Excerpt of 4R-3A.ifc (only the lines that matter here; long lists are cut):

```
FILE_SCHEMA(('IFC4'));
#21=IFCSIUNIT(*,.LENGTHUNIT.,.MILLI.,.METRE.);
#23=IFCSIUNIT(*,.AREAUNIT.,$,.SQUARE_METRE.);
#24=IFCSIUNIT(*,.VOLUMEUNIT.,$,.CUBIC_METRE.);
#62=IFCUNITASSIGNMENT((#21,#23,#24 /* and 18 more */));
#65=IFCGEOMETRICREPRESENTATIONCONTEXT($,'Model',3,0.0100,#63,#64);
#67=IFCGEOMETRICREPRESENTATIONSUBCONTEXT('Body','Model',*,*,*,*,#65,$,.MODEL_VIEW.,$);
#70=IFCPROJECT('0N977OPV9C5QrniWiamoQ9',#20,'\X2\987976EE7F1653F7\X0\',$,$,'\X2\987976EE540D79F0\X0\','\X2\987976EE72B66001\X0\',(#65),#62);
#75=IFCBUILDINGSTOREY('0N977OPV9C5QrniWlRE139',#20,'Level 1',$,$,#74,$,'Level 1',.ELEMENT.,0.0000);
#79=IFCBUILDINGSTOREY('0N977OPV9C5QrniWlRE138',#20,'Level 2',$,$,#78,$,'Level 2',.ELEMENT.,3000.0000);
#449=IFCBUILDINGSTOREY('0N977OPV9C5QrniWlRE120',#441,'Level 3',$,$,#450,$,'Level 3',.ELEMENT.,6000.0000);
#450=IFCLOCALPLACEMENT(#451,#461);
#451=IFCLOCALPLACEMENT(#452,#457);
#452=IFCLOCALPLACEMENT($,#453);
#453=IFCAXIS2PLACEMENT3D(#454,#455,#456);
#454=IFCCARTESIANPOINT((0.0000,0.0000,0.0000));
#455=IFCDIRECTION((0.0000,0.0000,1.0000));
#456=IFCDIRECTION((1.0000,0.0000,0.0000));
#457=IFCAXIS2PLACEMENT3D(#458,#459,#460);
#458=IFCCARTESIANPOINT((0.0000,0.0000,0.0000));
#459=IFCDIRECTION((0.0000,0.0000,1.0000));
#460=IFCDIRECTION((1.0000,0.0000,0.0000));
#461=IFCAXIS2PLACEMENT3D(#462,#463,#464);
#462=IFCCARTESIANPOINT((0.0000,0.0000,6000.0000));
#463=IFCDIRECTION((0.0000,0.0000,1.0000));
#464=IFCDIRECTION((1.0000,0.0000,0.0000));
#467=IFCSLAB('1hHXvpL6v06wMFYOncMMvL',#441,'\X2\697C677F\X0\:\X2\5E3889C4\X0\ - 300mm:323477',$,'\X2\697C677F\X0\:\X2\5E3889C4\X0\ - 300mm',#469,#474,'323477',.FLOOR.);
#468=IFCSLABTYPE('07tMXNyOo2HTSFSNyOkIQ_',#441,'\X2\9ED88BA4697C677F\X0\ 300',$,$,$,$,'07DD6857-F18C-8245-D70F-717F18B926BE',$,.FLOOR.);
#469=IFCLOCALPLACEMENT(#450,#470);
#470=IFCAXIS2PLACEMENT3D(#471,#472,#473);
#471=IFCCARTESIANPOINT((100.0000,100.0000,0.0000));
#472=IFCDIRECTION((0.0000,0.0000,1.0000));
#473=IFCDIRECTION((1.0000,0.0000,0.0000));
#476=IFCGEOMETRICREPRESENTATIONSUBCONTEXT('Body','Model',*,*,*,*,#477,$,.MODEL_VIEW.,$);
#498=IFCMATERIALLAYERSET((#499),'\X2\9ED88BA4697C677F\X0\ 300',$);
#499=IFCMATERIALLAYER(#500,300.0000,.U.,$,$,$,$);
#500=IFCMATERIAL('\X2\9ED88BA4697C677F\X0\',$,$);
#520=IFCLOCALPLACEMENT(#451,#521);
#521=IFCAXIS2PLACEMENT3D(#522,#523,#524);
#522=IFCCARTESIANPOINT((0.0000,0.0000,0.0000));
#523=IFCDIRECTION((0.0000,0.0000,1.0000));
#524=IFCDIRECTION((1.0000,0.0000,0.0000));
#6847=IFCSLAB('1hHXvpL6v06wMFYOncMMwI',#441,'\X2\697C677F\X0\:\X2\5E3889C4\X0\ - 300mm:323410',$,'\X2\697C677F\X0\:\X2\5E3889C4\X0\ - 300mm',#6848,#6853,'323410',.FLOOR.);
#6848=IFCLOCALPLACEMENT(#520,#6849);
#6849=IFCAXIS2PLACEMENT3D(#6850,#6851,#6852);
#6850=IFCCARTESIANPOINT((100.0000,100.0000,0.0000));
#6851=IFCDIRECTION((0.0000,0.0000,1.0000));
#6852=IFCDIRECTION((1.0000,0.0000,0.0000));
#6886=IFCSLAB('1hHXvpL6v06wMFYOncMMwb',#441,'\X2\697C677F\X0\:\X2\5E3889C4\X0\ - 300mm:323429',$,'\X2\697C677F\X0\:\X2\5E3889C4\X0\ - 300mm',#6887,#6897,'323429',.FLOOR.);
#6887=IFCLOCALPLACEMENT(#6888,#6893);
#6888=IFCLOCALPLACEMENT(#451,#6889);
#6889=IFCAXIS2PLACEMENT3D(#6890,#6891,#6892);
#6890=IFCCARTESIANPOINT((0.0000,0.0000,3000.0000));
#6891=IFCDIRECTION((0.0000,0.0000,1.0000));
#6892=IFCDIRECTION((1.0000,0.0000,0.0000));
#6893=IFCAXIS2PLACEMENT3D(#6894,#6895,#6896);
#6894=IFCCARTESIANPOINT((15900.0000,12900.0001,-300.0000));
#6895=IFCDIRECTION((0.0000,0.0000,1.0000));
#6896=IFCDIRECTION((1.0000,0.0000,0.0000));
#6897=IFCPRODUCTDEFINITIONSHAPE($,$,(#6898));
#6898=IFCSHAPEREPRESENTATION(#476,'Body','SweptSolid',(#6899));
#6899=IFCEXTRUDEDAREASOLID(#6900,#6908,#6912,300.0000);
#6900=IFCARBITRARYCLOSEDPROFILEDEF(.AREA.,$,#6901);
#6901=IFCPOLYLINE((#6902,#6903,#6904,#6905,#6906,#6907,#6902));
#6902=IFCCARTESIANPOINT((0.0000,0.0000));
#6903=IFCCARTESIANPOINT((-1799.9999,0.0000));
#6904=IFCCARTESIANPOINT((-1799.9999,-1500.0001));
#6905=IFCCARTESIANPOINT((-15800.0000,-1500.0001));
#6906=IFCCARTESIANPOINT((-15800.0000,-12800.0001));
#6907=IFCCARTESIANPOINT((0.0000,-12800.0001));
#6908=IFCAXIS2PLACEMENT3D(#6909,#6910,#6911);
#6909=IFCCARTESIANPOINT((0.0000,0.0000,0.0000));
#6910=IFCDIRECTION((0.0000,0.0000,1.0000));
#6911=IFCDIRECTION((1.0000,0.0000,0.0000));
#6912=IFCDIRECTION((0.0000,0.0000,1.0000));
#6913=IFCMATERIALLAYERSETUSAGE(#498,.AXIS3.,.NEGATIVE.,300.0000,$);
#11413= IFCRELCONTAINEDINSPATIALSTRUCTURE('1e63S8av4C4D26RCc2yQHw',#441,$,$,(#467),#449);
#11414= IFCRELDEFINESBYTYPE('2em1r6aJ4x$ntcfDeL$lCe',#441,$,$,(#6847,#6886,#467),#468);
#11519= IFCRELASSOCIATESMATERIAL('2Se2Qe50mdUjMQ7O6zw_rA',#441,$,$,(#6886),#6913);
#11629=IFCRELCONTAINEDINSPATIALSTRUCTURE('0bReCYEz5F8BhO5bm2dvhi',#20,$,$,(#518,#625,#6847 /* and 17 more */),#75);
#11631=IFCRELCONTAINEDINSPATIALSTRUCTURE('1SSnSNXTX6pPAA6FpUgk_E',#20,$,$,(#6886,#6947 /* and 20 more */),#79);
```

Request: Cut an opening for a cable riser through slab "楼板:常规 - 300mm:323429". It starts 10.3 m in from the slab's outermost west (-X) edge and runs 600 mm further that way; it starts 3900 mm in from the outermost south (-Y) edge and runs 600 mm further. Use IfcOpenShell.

```python
import numpy as np
import ifcopenshell
import ifcopenshell.api.feature
import ifcopenshell.api.geometry
import ifcopenshell.api.root
import ifcopenshell.geom
import ifcopenshell.util.placement
import ifcopenshell.util.representation
import ifcopenshell.util.shape
import ifcopenshell.util.unit

model = ifcopenshell.open("4R-3A.ifc")
unit_scale = ifcopenshell.util.unit.calculate_unit_scale(model)
settings = ifcopenshell.geom.settings()


def volume(element):
    """Net volume in cubic metres, openings subtracted."""
    shape = ifcopenshell.geom.create_shape(settings, element)
    return ifcopenshell.util.shape.get_volume(shape.geometry)


slab = model.by_guid("1hHXvpL6v06wMFYOncMMwb")
before = volume(slab)

# Extent in the slab's own axes, in metres. The edges named are its -X and -Y sides.
slab_shape = ifcopenshell.geom.create_shape(settings, slab)
vertices = ifcopenshell.util.shape.get_vertices(slab_shape.geometry)
x_min, y_min, bottom = vertices.min(axis=0)
top = vertices[:, 2].max()

opening = ifcopenshell.api.root.create_entity(model, ifc_class="IfcOpeningElement", name="Cable riser opening", predefined_type="OPENING")
context = ifcopenshell.util.representation.get_context(model, "Model", "Body", "MODEL_VIEW")
width, depth = 0.6, 0.6
outline = [(0.0, 0.0), (width, 0.0), (width, depth), (0.0, depth), (0.0, 0.0)]
# Overshoot both faces by 50 mm so the cut is clean.
shape = ifcopenshell.api.geometry.add_slab_representation(
    model, context=context, depth=top - bottom + 0.1, polyline=outline
)
ifcopenshell.api.geometry.assign_representation(model, product=opening, representation=shape)

matrix = ifcopenshell.util.placement.get_local_placement(slab.ObjectPlacement)
matrix[:, 3] = matrix @ np.append(np.array([x_min + 10.3, y_min + 3.9, bottom - 0.05]) / unit_scale, 1.0)
ifcopenshell.api.geometry.edit_object_placement(model, product=opening, matrix=matrix, is_si=False)
ifcopenshell.api.feature.add_feature(model, feature=opening, element=slab)

after = volume(slab)

print(f"slab volume {before:.3f} -> {after:.3f} m3")

model.write("4R-3A_v2.ifc")
```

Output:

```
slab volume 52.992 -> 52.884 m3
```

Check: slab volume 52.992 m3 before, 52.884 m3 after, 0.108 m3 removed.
